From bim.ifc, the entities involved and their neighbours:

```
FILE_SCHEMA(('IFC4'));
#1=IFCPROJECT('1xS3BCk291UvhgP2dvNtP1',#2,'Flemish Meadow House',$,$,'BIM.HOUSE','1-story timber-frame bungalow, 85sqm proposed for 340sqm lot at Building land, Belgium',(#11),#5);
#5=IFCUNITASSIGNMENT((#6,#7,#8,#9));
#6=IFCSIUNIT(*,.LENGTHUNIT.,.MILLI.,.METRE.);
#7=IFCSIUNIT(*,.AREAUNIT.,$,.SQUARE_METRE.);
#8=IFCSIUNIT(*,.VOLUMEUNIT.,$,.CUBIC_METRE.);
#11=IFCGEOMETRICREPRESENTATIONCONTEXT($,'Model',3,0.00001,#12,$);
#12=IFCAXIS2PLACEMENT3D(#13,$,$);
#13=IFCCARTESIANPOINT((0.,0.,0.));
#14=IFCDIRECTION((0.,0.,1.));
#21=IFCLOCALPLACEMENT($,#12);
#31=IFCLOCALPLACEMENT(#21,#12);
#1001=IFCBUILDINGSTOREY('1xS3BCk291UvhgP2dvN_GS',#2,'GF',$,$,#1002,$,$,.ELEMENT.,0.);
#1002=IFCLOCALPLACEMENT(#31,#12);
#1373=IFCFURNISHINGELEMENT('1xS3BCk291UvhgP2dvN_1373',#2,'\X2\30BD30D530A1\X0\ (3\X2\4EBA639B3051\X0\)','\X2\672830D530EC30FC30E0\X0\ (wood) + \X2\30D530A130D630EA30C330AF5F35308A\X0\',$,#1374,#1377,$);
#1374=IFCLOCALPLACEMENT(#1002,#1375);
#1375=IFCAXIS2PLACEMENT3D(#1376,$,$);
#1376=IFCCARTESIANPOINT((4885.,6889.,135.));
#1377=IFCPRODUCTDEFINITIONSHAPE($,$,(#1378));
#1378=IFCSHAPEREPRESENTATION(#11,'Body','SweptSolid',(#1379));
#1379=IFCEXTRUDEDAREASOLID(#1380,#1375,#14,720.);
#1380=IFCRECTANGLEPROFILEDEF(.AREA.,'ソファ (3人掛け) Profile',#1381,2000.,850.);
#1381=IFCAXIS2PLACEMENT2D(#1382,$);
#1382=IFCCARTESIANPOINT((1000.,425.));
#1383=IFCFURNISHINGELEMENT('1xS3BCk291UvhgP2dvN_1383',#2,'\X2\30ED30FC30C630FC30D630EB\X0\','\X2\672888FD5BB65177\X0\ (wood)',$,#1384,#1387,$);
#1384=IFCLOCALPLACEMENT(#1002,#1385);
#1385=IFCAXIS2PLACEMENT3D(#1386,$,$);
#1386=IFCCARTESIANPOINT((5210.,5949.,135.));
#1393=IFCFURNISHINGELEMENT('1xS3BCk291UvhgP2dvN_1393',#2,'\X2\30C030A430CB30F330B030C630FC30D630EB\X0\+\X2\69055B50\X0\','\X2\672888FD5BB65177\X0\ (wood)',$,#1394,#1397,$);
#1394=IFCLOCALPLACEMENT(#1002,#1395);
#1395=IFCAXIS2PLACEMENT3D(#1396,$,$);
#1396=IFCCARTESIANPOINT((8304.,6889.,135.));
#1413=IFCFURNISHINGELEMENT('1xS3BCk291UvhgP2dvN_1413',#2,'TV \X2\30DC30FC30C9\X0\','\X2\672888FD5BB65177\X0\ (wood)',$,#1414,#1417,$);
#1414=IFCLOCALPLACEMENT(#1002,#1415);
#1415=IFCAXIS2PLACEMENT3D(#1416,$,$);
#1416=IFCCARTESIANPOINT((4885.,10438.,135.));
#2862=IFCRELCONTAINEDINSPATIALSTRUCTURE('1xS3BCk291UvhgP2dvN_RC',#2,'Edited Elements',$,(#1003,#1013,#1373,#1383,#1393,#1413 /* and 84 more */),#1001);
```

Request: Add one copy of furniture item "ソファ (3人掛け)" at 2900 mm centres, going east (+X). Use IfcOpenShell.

```python
import numpy as np
import ifcopenshell
import ifcopenshell.api.geometry
import ifcopenshell.api.root
import ifcopenshell.util.element
import ifcopenshell.util.placement

model = ifcopenshell.open("bim.ifc")


def reuse_history(source, copy):
    """copy_class also copies each property set's owner history, people and application; keep the originals."""
    for rel in copy.IsDefinedBy:
        if rel.is_a("IfcRelDefinesByProperties") and (history := rel.RelatingPropertyDefinition.OwnerHistory):
            rel.RelatingPropertyDefinition.OwnerHistory = source.OwnerHistory
            ifcopenshell.util.element.remove_deep2(model, history)


source = model.by_guid("1xS3BCk291UvhgP2dvN_1373")
base = ifcopenshell.util.placement.get_local_placement(source.ObjectPlacement)
step = np.array([1.0, 0.0, 0.0]) * 2900.0

for i in range(1, 2):
    copy = ifcopenshell.api.root.copy_class(model, product=source)
    copy.Representation = ifcopenshell.util.element.copy_deep(
        model, source.Representation, exclude=["IfcGeometricRepresentationContext", "IfcRepresentationMap"]
    )
    reuse_history(source, copy)
    matrix = base.copy()
    matrix[:3, 3] += i * step
    print("added at", matrix[:3, 3].round(3) + 0.0)
    ifcopenshell.api.geometry.edit_object_placement(model, product=copy, matrix=matrix, is_si=False)

model.write("bim_v2.ifc")
```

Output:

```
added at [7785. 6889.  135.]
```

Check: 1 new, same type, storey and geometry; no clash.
